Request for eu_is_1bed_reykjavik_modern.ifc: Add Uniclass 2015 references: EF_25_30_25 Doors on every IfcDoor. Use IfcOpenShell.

First a look at what the model holds.

```python
import ifcopenshell

model = ifcopenshell.open("eu_is_1bed_reykjavik_modern.ifc")
print(model.schema)
print("classifications:", [c.Name for c in model.by_type("IfcClassification")])
for ifc_class in ("IfcDoor", "IfcRoof", "IfcStair", "IfcWall", "IfcWindow"):
    print(ifc_class, len(model.by_type(ifc_class)))
```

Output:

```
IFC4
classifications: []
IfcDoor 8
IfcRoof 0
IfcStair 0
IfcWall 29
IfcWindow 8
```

```python
import ifcopenshell
import ifcopenshell.api.classification

model = ifcopenshell.open("eu_is_1bed_reykjavik_modern.ifc")

system = ifcopenshell.api.classification.add_classification(model, classification="Uniclass 2015")

codes = {
    "IfcDoor": ("EF_25_30_25", "Doors"),
}
for ifc_class, (code, name) in codes.items():
    products = model.by_type(ifc_class)
    ifcopenshell.api.classification.add_reference(
        model, products=products, classification=system, identification=code, name=name
    )
    print(code, len(products))

model.write("eu_is_1bed_reykjavik_modern_updated.ifc")
```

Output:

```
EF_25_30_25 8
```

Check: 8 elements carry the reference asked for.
